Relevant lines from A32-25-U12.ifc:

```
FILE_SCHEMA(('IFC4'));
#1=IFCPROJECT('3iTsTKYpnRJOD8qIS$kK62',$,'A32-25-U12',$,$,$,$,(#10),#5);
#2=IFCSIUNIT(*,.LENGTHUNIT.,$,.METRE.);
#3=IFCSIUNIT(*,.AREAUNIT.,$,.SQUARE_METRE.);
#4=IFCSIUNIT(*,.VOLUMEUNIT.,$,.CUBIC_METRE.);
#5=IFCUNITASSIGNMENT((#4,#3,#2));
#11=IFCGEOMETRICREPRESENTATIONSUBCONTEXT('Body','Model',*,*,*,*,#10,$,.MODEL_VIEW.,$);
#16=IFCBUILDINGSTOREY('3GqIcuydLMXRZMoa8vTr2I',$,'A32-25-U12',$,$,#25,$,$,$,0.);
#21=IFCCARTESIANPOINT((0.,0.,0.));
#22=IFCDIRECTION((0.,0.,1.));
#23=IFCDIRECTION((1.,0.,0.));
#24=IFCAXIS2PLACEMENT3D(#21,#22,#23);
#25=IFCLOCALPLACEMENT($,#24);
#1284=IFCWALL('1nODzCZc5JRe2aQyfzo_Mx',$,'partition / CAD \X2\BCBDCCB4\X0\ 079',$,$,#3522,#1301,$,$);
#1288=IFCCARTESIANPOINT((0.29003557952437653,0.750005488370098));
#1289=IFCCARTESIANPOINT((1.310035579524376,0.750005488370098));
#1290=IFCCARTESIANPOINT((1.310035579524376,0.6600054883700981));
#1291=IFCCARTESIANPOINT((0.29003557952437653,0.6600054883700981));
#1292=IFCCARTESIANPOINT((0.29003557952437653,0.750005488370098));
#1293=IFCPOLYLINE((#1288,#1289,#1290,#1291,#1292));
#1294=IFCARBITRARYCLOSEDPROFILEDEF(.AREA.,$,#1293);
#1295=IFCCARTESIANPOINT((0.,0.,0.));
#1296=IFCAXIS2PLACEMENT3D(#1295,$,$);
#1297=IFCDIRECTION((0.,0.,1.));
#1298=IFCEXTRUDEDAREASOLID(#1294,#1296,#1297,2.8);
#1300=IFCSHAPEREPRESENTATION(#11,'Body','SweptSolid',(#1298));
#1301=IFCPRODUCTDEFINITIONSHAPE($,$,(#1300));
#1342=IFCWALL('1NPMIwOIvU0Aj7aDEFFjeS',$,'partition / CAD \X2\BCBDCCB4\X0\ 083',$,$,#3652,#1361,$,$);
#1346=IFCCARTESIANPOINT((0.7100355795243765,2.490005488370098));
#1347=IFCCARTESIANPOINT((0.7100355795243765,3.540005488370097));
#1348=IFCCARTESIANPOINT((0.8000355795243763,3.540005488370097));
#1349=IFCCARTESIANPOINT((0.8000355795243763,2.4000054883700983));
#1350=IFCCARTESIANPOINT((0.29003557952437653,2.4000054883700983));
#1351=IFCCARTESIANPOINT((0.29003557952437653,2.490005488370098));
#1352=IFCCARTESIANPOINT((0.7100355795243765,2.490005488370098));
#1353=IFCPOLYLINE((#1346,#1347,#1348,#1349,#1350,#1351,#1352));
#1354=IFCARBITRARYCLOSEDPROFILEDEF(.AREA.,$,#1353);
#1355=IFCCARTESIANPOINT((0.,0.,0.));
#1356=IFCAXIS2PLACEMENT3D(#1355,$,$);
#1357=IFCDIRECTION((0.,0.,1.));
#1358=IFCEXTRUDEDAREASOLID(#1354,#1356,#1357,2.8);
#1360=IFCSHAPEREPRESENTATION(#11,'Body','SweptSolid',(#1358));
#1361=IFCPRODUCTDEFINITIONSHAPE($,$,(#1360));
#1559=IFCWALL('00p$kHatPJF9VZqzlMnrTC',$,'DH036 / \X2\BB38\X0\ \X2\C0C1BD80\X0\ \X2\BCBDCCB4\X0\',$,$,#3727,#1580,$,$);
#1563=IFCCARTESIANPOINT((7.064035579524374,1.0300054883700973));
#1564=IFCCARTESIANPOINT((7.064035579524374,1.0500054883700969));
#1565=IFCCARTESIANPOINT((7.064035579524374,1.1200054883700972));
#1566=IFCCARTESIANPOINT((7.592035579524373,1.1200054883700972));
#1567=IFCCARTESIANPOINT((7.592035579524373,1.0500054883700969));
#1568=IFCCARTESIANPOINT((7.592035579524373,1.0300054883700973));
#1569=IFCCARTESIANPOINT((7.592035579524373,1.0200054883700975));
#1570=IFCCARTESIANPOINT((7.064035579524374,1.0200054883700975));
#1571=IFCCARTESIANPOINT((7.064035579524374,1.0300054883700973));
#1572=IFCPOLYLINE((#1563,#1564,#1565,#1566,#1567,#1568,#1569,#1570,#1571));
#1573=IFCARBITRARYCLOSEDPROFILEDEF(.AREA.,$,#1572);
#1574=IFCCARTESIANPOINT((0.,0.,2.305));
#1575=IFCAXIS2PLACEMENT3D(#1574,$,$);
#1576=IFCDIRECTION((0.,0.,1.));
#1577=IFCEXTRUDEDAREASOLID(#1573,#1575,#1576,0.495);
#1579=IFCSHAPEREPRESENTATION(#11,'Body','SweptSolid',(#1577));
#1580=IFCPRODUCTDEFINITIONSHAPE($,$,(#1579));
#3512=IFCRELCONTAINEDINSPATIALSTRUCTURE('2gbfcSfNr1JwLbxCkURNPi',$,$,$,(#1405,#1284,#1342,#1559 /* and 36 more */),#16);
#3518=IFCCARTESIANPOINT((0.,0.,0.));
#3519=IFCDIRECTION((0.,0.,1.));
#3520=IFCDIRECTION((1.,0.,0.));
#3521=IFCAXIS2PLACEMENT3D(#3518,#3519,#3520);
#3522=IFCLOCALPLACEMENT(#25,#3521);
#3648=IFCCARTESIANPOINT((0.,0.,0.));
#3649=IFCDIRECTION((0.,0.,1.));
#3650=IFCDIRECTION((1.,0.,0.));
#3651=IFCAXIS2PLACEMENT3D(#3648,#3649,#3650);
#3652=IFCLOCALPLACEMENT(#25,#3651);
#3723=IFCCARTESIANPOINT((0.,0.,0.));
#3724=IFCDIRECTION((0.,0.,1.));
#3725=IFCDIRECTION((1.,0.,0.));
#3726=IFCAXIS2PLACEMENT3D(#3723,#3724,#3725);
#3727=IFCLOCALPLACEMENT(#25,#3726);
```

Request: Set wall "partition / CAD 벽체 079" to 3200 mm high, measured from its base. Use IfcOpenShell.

```python
import ifcopenshell
import ifcopenshell.geom
import ifcopenshell.util.representation
import ifcopenshell.util.shape

model = ifcopenshell.open("A32-25-U12.ifc")
settings = ifcopenshell.geom.settings()


def volume(element):
    """Net volume in cubic metres, openings subtracted."""
    shape = ifcopenshell.geom.create_shape(settings, element)
    return ifcopenshell.util.shape.get_volume(shape.geometry)


wall = model.by_guid("1nODzCZc5JRe2aQyfzo_Mx")
before = volume(wall)

body = ifcopenshell.util.representation.get_representation(wall, "Model", "Body")
solid = body.Items[0]
old_height = solid.Depth
solid.Depth = 3.2
after = volume(wall)

print(f"height {old_height:g} -> {solid.Depth:g}, volume {before:.3f} -> {after:.3f} m3")

model.write("A32-25-U12-out.ifc")
```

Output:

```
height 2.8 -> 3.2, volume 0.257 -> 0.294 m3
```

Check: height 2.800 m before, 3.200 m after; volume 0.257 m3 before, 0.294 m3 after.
